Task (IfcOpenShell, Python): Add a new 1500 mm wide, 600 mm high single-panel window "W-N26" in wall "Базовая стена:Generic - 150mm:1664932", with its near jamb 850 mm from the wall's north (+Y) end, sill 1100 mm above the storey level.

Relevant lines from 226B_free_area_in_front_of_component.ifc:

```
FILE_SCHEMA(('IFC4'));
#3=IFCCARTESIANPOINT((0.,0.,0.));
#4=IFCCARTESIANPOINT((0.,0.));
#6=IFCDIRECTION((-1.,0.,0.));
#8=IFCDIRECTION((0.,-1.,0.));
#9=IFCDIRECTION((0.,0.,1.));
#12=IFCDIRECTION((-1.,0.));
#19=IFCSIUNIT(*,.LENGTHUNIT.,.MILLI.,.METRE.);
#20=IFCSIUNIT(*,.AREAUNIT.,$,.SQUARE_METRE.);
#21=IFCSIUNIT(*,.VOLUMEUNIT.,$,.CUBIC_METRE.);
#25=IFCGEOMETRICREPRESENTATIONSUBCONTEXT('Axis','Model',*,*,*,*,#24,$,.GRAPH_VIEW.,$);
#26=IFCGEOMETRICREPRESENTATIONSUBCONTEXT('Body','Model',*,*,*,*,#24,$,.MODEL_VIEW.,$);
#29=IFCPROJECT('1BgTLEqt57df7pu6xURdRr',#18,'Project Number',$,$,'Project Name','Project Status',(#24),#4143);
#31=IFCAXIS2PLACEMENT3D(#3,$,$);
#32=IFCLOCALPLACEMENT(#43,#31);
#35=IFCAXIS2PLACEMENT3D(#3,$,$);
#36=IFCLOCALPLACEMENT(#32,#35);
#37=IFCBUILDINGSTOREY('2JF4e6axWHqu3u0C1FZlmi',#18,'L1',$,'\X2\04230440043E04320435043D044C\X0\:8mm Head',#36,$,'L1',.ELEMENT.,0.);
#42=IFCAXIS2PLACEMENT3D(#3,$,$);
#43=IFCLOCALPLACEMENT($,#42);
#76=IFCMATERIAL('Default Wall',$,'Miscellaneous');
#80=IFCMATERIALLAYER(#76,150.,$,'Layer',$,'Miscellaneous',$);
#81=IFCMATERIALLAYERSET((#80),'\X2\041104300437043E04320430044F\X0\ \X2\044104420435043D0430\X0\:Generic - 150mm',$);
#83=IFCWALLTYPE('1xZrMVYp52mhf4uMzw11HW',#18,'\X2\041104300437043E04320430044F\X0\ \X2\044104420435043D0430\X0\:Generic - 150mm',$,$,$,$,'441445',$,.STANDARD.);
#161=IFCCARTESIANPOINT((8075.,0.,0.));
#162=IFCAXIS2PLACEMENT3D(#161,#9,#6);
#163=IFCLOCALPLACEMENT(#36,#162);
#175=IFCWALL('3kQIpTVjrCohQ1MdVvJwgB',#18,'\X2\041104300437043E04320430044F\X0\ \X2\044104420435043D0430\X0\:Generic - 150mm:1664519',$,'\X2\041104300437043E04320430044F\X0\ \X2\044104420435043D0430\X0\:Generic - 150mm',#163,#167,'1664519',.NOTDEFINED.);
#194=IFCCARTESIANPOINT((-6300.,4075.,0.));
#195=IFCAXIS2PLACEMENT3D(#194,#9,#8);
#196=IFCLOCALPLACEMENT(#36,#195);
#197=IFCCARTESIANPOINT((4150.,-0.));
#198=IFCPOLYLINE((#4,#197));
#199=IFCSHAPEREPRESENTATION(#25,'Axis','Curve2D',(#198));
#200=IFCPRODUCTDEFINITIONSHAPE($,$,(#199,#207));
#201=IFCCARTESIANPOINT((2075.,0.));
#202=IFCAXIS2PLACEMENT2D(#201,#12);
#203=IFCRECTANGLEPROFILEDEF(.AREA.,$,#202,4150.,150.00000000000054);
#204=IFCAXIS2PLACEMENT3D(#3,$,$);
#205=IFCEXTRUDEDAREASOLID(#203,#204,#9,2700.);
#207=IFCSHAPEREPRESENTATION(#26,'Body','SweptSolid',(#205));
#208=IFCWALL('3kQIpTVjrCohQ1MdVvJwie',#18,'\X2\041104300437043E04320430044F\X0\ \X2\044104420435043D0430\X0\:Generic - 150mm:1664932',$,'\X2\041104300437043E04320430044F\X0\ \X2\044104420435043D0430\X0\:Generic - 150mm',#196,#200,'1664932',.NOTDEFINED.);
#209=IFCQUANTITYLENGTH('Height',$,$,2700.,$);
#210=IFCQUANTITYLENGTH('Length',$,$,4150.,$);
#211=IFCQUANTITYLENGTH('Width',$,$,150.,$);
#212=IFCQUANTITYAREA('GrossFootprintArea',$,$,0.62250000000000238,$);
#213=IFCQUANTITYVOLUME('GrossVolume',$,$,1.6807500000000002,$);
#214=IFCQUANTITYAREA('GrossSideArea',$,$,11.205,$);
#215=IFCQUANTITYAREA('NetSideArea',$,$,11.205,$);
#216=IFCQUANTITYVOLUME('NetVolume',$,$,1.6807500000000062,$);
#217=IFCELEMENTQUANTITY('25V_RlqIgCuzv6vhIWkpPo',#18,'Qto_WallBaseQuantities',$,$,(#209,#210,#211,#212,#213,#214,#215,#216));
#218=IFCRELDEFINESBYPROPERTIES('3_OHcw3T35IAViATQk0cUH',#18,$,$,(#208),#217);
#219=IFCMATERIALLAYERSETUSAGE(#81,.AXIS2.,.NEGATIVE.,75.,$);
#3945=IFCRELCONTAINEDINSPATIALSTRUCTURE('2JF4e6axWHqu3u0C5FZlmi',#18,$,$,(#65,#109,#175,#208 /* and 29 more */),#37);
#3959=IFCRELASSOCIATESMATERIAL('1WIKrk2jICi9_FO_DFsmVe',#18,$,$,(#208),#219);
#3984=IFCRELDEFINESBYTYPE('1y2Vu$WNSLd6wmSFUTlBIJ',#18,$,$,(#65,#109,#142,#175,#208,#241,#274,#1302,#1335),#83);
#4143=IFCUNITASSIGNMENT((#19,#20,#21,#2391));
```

```python
import numpy as np
import ifcopenshell
import ifcopenshell.api.feature
import ifcopenshell.api.geometry
import ifcopenshell.api.pset
import ifcopenshell.api.root
import ifcopenshell.api.spatial
import ifcopenshell.geom
import ifcopenshell.util.element
import ifcopenshell.util.placement
import ifcopenshell.util.representation
import ifcopenshell.util.shape
import ifcopenshell.util.unit

model = ifcopenshell.open("226B_free_area_in_front_of_component.ifc")
unit_scale = ifcopenshell.util.unit.calculate_unit_scale(model)
area_scale = ifcopenshell.util.unit.calculate_unit_scale(model, "AREAUNIT")
volume_scale = ifcopenshell.util.unit.calculate_unit_scale(model, "VOLUMEUNIT")
settings = ifcopenshell.geom.settings()


def volume(element):
    """Net volume in cubic metres, openings subtracted."""
    shape = ifcopenshell.geom.create_shape(settings, element)
    return ifcopenshell.util.shape.get_volume(shape.geometry)


wall = model.by_guid("3kQIpTVjrCohQ1MdVvJwie")
storey = ifcopenshell.util.element.get_container(wall, ifc_class="IfcBuildingStorey")
context = ifcopenshell.util.representation.get_context(model, "Model", "Body", "MODEL_VIEW")
before = volume(wall)

width, height, from_end, sill = 1.5, 0.6, 0.85, 1.1  # metres

# The wall runs along its own X axis, and the end named is its -X end.
wall_shape = ifcopenshell.geom.create_shape(settings, wall)
x, y, z = ifcopenshell.util.shape.get_vertices(wall_shape.geometry).T
start = x.min() + from_end
face, thickness = float(y.min()), float(y.max() - y.min())
wall_matrix = ifcopenshell.util.placement.get_local_placement(wall.ObjectPlacement)
level = ifcopenshell.util.placement.get_local_placement(storey.ObjectPlacement)[2, 3]


def in_wall(x, y):
    """Placement at x, y metres in the wall's axes, at sill height."""
    matrix = wall_matrix.copy()
    matrix[:, 3] = wall_matrix @ np.array([x / unit_scale, y / unit_scale, 0.0, 1.0])
    matrix[2, 3] = level + sill / unit_scale
    return matrix


# Opening: a box that overshoots both wall faces by 50 mm.
opening = ifcopenshell.api.root.create_entity(model, ifc_class="IfcOpeningElement", predefined_type="OPENING")
box = ifcopenshell.api.geometry.add_wall_representation(
    model, context=context, length=width, height=height, thickness=thickness + 0.1
)
ifcopenshell.api.geometry.assign_representation(model, product=opening, representation=box)
ifcopenshell.api.geometry.edit_object_placement(model, product=opening, matrix=in_wall(start, face - 0.05), is_si=False)
ifcopenshell.api.feature.add_feature(model, feature=opening, element=wall)

window = ifcopenshell.api.root.create_entity(model, ifc_class="IfcWindow", name="W-N26", predefined_type="WINDOW")
window.OverallWidth, window.OverallHeight = width / unit_scale, height / unit_scale
window.PartitioningType = "SINGLE_PANEL"
body = ifcopenshell.api.geometry.add_window_representation(
    model,
    context=context,
    overall_width=window.OverallWidth,
    overall_height=window.OverallHeight,
    partition_type="SINGLE_PANEL",
)
ifcopenshell.api.geometry.assign_representation(model, product=window, representation=body)
ifcopenshell.api.spatial.assign_container(model, products=[window], relating_structure=storey)
ifcopenshell.api.feature.add_filling(model, opening=opening, element=window)

# Centre the window in the wall's thickness.
ifcopenshell.api.geometry.edit_object_placement(model, product=window, matrix=in_wall(start, face), is_si=False)
window_shape = ifcopenshell.geom.create_shape(settings, window)
depth = ifcopenshell.util.shape.get_vertices(window_shape.geometry)[:, 1]
offset = face + thickness / 2 - (depth.min() + depth.max()) / 2
ifcopenshell.api.geometry.edit_object_placement(model, product=window, matrix=in_wall(start, offset), is_si=False)

after = volume(wall)

# Update the wall's stored quantities.
qto = model.by_id(ifcopenshell.util.element.get_pset(wall, "Qto_WallBaseQuantities", should_inherit=False)["id"])
ifcopenshell.api.pset.edit_qto(model, qto=qto, properties={
    "NetSideArea": after / thickness / area_scale,
    "NetVolume": after / volume_scale,
})

print(f"wall volume {before:.3f} -> {after:.3f} m3")

model.write("226B_free_area_in_front_of_component_edited.ifc")
```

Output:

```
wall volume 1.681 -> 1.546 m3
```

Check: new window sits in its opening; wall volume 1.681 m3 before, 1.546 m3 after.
